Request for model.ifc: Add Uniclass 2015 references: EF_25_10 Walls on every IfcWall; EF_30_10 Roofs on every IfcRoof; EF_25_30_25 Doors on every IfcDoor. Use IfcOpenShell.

First a look at what the model holds.

```python
import ifcopenshell

model = ifcopenshell.open("model.ifc")
print(model.schema)
print("classifications:", [c.Name for c in model.by_type("IfcClassification")])
for ifc_class in ("IfcDoor", "IfcRoof", "IfcStair", "IfcWall", "IfcWindow"):
    print(ifc_class, len(model.by_type(ifc_class)))
```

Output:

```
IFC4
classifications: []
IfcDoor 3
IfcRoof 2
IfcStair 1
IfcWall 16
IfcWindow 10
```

```python
import ifcopenshell
import ifcopenshell.api.classification

model = ifcopenshell.open("model.ifc")

system = ifcopenshell.api.classification.add_classification(model, classification="Uniclass 2015")

codes = {
    "IfcWall": ("EF_25_10", "Walls"),
    "IfcRoof": ("EF_30_10", "Roofs"),
    "IfcDoor": ("EF_25_30_25", "Doors"),
}
for ifc_class, (code, name) in codes.items():
    products = model.by_type(ifc_class)
    ifcopenshell.api.classification.add_reference(
        model, products=products, classification=system, identification=code, name=name
    )
    print(code, len(products))

model.write("model_edited.ifc")
```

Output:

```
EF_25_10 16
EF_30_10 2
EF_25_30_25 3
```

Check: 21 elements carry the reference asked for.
